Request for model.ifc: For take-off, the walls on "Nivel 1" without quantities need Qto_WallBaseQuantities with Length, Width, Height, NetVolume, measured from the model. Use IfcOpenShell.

First a look at what the model holds.

```python
import ifcopenshell
import ifcopenshell.util.element
import ifcopenshell.util.unit

model = ifcopenshell.open("model.ifc")
print(model.schema)
for unit_type in ("LENGTHUNIT", "AREAUNIT", "VOLUMEUNIT"):
    print(unit_type, ifcopenshell.util.unit.calculate_unit_scale(model, unit_type))
storey = next(s for s in model.by_type("IfcBuildingStorey") if s.Name == "Nivel 1")
walls = [e for e in ifcopenshell.util.element.get_decomposition(storey) if e.is_a("IfcWall")]
for e in sorted(walls, key=lambda e: e.id()):
    print(e.id(), e.is_a(), e.Name, list(ifcopenshell.util.element.get_psets(e, qtos_only=True)), sep=" | ")
```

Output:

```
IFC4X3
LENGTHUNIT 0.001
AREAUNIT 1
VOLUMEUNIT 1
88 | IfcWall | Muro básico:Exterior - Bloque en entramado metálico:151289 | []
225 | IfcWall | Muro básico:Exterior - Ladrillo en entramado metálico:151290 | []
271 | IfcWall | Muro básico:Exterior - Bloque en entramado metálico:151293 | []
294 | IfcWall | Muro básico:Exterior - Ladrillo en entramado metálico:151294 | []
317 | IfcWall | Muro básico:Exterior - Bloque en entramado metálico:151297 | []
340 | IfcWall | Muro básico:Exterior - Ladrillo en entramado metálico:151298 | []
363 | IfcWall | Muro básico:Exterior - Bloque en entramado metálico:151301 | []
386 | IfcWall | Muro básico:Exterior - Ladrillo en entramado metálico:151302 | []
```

```python
import ifcopenshell
import ifcopenshell.api.pset
import ifcopenshell.geom
import ifcopenshell.util.element
import ifcopenshell.util.shape
import ifcopenshell.util.unit

model = ifcopenshell.open("model.ifc")
unit_scale = ifcopenshell.util.unit.calculate_unit_scale(model)
volume_scale = ifcopenshell.util.unit.calculate_unit_scale(model, "VOLUMEUNIT")
settings = ifcopenshell.geom.settings()

storey = next(s for s in model.by_type("IfcBuildingStorey") if s.Name == "Nivel 1")
walls = [e for e in ifcopenshell.util.element.get_decomposition(storey) if e.is_a("IfcWall")]

for e in sorted(walls, key=lambda e: e.id()):
    if ifcopenshell.util.element.get_psets(e, qtos_only=True, should_inherit=False):
        continue
    # Geometry comes back in metres, in the element's own axes.
    shape = ifcopenshell.geom.create_shape(settings, e)
    values = {
        "Length": ifcopenshell.util.shape.get_x(shape.geometry) / unit_scale,
        "Width": ifcopenshell.util.shape.get_y(shape.geometry) / unit_scale,
        "Height": ifcopenshell.util.shape.get_z(shape.geometry) / unit_scale,
        "NetVolume": ifcopenshell.util.shape.get_volume(shape.geometry) / volume_scale,
    }
    qto = ifcopenshell.api.pset.add_qto(model, product=e, name="Qto_WallBaseQuantities")
    ifcopenshell.api.pset.edit_qto(model, qto=qto, properties=values)
    print(e.id(), {k: round(v, 3) for k, v in values.items()})

model.write("model_rev.ifc")
```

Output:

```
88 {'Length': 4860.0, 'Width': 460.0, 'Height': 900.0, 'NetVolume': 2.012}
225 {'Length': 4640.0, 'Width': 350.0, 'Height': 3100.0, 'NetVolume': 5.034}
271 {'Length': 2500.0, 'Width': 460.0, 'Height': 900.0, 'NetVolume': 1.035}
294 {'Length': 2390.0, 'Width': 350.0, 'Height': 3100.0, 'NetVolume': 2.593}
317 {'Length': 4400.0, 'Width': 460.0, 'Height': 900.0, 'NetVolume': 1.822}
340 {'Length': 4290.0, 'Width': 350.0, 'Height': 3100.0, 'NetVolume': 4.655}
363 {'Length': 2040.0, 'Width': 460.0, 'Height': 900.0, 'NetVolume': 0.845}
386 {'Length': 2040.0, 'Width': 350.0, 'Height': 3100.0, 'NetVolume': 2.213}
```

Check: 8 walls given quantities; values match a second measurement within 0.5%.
